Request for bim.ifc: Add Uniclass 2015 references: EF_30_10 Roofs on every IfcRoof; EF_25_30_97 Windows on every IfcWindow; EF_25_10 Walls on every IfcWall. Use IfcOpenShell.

First a look at what the model holds.

```python
import ifcopenshell

model = ifcopenshell.open("bim.ifc")
print(model.schema)
print("classifications:", [c.Name for c in model.by_type("IfcClassification")])
for ifc_class in ("IfcDoor", "IfcRoof", "IfcStair", "IfcWall", "IfcWindow"):
    print(ifc_class, len(model.by_type(ifc_class)))
```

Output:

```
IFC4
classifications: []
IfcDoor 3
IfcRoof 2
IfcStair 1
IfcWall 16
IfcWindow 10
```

```python
import ifcopenshell
import ifcopenshell.api.classification

model = ifcopenshell.open("bim.ifc")

system = ifcopenshell.api.classification.add_classification(model, classification="Uniclass 2015")

codes = {
    "IfcRoof": ("EF_30_10", "Roofs"),
    "IfcWindow": ("EF_25_30_97", "Windows"),
    "IfcWall": ("EF_25_10", "Walls"),
}
for ifc_class, (code, name) in codes.items():
    products = model.by_type(ifc_class)
    ifcopenshell.api.classification.add_reference(
        model, products=products, classification=system, identification=code, name=name
    )
    print(code, len(products))

model.write("bim_v2.ifc")
```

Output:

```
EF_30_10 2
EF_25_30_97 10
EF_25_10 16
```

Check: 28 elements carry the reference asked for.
